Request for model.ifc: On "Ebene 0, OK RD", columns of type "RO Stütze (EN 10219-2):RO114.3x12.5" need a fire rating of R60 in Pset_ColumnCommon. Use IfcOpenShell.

First a look at what the model holds.

```python
import ifcopenshell
import ifcopenshell.util.element

model = ifcopenshell.open("model.ifc")
print(model.schema)
storey = next(s for s in model.by_type("IfcBuildingStorey") if s.Name == "Ebene 0, OK RD")
columns = [e for e in ifcopenshell.util.element.get_decomposition(storey) if e.is_a("IfcColumn")]
seen = {}
for e in columns:
    element_type = ifcopenshell.util.element.get_type(e)
    key = (element_type.Name if element_type != e and element_type else None, ifcopenshell.util.element.get_pset(e, "Pset_ColumnCommon", "FireRating"))
    seen[key] = seen.get(key, 0) + 1
for (name, value), count in sorted(seen.items(), key=str):
    print(count, "x", name, "|", value)
```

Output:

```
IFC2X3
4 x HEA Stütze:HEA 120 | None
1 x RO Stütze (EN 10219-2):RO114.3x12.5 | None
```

```python
import ifcopenshell
import ifcopenshell.api.pset
import ifcopenshell.util.element

model = ifcopenshell.open("model.ifc")

storey = next(s for s in model.by_type("IfcBuildingStorey") if s.Name == "Ebene 0, OK RD")
columns = [e for e in ifcopenshell.util.element.get_decomposition(storey) if e.is_a("IfcColumn")]

count = 0
for e in columns:
    element_type = ifcopenshell.util.element.get_type(e)
    if element_type in (None, e) or element_type.Name != "RO Stütze (EN 10219-2):RO114.3x12.5":
        continue
    # add_pset returns the element's existing set when there is one.
    pset = ifcopenshell.api.pset.add_pset(model, product=e, name="Pset_ColumnCommon")
    ifcopenshell.api.pset.edit_pset(model, pset=pset, properties={"FireRating": "R60"})
    count += 1

print(count, "columns updated")

model.write("model_updated.ifc")
```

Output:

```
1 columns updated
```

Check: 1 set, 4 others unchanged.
